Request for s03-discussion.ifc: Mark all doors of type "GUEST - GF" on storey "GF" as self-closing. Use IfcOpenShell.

First a look at what the model holds.

```python
import ifcopenshell
import ifcopenshell.util.element

model = ifcopenshell.open("s03-discussion.ifc")
print(model.schema)
storey = next(s for s in model.by_type("IfcBuildingStorey") if s.Name == "GF")
doors = [e for e in ifcopenshell.util.element.get_decomposition(storey) if e.is_a("IfcDoor")]
seen = {}
for e in doors:
    element_type = ifcopenshell.util.element.get_type(e)
    key = (element_type.Name if element_type != e and element_type else None, ifcopenshell.util.element.get_pset(e, "Pset_DoorCommon", "SelfClosing"))
    seen[key] = seen.get(key, 0) + 1
for (name, value), count in sorted(seen.items(), key=str):
    print(count, "x", name, "|", value)
```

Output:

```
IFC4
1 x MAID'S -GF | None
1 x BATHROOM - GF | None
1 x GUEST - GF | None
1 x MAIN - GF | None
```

```python
import ifcopenshell
import ifcopenshell.api.pset
import ifcopenshell.util.element

model = ifcopenshell.open("s03-discussion.ifc")

storey = next(s for s in model.by_type("IfcBuildingStorey") if s.Name == "GF")
doors = [e for e in ifcopenshell.util.element.get_decomposition(storey) if e.is_a("IfcDoor")]

count = 0
for e in doors:
    element_type = ifcopenshell.util.element.get_type(e)
    if element_type in (None, e) or element_type.Name != "GUEST - GF":
        continue
    # add_pset returns the element's existing set when there is one.
    pset = ifcopenshell.api.pset.add_pset(model, product=e, name="Pset_DoorCommon")
    ifcopenshell.api.pset.edit_pset(model, pset=pset, properties={"SelfClosing": True})
    count += 1

print(count, "doors updated")

model.write("s03-discussion_rev.ifc")
```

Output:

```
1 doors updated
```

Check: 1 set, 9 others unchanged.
